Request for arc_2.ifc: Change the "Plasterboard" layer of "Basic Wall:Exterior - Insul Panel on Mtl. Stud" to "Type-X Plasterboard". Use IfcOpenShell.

First a look at what the model holds.

```python
import ifcopenshell
import ifcopenshell.util.element

model = ifcopenshell.open("arc_2.ifc")
print(model.schema)
for layer_set in model.by_type("IfcMaterialLayerSet"):
    if layer_set.LayerSetName == "Basic Wall:Exterior - Insul Panel on Mtl. Stud":
        for layer in layer_set.MaterialLayers:
            print(layer.id(), layer.Material and layer.Material.Name, layer.LayerThickness, sep=" | ")
        print(len(ifcopenshell.util.element.get_elements_by_material(model, layer_set)), "elements and types use it")
print(sorted(m.Name for m in model.by_type("IfcMaterial") if m.Name)[:60])
```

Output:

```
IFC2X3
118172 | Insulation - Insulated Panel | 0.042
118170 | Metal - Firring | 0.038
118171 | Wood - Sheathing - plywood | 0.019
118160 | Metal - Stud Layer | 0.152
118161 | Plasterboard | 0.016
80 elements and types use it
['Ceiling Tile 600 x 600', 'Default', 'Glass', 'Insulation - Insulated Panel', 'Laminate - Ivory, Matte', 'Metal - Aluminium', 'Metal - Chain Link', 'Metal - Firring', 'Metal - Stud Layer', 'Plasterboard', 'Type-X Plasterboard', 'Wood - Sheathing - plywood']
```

```python
import ifcopenshell
import ifcopenshell.api.material

model = ifcopenshell.open("arc_2.ifc")

layer_set = next(s for s in model.by_type("IfcMaterialLayerSet") if s.LayerSetName == "Basic Wall:Exterior - Insul Panel on Mtl. Stud")
layer = next(l for l in layer_set.MaterialLayers if l.Material and l.Material.Name == "Plasterboard")
material = next(m for m in model.by_type("IfcMaterial") if m.Name == "Type-X Plasterboard")

# Point this one layer at the other material; renaming the old one would change it everywhere.
ifcopenshell.api.material.edit_layer(model, layer=layer, attributes={}, material=material)

print([l.Material.Name if l.Material else None for l in layer_set.MaterialLayers])

model.write("arc_2_rev.ifc")
```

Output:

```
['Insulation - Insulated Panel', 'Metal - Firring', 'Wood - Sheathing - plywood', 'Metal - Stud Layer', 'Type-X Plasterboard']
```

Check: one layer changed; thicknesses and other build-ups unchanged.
